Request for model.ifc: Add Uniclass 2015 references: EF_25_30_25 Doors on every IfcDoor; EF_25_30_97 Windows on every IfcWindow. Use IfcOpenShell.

First a look at what the model holds.

```python
import ifcopenshell

model = ifcopenshell.open("model.ifc")
print(model.schema)
print("classifications:", [c.Name for c in model.by_type("IfcClassification")])
for ifc_class in ("IfcDoor", "IfcRoof", "IfcStair", "IfcWall", "IfcWindow"):
    print(ifc_class, len(model.by_type(ifc_class)))
```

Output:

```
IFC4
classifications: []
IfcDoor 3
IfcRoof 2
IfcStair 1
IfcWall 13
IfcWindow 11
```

```python
import ifcopenshell
import ifcopenshell.api.classification

model = ifcopenshell.open("model.ifc")

system = ifcopenshell.api.classification.add_classification(model, classification="Uniclass 2015")

codes = {
    "IfcDoor": ("EF_25_30_25", "Doors"),
    "IfcWindow": ("EF_25_30_97", "Windows"),
}
for ifc_class, (code, name) in codes.items():
    products = model.by_type(ifc_class)
    ifcopenshell.api.classification.add_reference(
        model, products=products, classification=system, identification=code, name=name
    )
    print(code, len(products))

model.write("model_updated.ifc")
```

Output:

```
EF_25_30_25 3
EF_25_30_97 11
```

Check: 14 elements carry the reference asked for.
